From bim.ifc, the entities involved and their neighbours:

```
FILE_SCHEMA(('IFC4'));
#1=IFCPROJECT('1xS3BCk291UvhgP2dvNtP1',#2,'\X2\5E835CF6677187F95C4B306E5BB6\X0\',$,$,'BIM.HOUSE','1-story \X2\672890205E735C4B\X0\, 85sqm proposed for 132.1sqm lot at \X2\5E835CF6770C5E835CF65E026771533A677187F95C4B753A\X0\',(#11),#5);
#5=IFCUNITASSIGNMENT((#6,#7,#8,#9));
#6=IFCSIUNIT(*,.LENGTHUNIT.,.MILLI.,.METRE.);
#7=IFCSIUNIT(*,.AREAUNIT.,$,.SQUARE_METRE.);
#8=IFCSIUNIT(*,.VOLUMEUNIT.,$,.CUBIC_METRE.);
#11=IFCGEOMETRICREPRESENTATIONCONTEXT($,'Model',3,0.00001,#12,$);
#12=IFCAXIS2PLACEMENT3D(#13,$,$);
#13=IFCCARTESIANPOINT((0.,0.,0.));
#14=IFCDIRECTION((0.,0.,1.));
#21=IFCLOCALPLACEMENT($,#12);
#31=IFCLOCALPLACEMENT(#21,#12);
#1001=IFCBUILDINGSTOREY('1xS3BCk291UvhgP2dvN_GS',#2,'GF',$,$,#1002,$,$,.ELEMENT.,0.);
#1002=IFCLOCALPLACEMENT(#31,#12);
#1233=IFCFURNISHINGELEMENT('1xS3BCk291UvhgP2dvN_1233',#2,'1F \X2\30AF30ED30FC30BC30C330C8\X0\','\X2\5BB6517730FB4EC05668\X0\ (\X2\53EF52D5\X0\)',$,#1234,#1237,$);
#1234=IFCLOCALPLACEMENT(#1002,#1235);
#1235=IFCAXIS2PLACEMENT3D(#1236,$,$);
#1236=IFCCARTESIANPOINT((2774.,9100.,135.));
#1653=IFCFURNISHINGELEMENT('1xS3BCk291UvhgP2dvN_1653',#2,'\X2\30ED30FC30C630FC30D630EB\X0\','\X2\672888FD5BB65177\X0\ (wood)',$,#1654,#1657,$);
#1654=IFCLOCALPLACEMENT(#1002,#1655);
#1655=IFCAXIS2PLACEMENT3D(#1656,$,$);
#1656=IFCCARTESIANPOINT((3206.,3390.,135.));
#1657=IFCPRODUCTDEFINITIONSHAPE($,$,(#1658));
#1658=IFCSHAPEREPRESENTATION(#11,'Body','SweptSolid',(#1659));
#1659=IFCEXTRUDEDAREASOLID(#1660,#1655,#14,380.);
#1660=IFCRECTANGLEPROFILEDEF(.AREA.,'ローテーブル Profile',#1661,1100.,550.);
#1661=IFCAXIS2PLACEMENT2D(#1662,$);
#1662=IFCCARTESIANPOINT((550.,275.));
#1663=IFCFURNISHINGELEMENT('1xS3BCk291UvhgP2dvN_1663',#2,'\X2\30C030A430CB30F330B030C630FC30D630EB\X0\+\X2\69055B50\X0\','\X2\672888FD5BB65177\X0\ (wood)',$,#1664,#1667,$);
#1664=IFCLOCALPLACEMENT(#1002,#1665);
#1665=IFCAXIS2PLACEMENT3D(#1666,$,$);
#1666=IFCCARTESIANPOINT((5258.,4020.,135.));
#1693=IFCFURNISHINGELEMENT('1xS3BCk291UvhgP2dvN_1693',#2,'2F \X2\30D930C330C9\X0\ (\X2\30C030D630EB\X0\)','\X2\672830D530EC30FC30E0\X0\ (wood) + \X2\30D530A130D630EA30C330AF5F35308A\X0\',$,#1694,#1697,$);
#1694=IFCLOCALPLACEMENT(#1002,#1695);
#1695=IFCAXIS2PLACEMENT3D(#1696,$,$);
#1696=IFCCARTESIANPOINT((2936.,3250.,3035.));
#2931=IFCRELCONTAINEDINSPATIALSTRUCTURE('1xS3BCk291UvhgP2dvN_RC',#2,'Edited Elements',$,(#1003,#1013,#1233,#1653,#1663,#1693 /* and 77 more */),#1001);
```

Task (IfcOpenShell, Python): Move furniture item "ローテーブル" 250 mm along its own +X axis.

```python
import ifcopenshell
import ifcopenshell.api.geometry
import ifcopenshell.util.placement
import ifcopenshell.util.unit

model = ifcopenshell.open("bim.ifc")
unit_scale = ifcopenshell.util.unit.calculate_unit_scale(model)

item = model.by_id(1653)
matrix = ifcopenshell.util.placement.get_local_placement(item.ObjectPlacement)
matrix[:3, 3] += matrix[:3, 0] * 0.25 / unit_scale
ifcopenshell.api.geometry.edit_object_placement(model, product=item, matrix=matrix, is_si=False)

print(ifcopenshell.util.placement.get_local_placement(item.ObjectPlacement).round(3) + 0.0)

model.write("bim-out.ifc")
```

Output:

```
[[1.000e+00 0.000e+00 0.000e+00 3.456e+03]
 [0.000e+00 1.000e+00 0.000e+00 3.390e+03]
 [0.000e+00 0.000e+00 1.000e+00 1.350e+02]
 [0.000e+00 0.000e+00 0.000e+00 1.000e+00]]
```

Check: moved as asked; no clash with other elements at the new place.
